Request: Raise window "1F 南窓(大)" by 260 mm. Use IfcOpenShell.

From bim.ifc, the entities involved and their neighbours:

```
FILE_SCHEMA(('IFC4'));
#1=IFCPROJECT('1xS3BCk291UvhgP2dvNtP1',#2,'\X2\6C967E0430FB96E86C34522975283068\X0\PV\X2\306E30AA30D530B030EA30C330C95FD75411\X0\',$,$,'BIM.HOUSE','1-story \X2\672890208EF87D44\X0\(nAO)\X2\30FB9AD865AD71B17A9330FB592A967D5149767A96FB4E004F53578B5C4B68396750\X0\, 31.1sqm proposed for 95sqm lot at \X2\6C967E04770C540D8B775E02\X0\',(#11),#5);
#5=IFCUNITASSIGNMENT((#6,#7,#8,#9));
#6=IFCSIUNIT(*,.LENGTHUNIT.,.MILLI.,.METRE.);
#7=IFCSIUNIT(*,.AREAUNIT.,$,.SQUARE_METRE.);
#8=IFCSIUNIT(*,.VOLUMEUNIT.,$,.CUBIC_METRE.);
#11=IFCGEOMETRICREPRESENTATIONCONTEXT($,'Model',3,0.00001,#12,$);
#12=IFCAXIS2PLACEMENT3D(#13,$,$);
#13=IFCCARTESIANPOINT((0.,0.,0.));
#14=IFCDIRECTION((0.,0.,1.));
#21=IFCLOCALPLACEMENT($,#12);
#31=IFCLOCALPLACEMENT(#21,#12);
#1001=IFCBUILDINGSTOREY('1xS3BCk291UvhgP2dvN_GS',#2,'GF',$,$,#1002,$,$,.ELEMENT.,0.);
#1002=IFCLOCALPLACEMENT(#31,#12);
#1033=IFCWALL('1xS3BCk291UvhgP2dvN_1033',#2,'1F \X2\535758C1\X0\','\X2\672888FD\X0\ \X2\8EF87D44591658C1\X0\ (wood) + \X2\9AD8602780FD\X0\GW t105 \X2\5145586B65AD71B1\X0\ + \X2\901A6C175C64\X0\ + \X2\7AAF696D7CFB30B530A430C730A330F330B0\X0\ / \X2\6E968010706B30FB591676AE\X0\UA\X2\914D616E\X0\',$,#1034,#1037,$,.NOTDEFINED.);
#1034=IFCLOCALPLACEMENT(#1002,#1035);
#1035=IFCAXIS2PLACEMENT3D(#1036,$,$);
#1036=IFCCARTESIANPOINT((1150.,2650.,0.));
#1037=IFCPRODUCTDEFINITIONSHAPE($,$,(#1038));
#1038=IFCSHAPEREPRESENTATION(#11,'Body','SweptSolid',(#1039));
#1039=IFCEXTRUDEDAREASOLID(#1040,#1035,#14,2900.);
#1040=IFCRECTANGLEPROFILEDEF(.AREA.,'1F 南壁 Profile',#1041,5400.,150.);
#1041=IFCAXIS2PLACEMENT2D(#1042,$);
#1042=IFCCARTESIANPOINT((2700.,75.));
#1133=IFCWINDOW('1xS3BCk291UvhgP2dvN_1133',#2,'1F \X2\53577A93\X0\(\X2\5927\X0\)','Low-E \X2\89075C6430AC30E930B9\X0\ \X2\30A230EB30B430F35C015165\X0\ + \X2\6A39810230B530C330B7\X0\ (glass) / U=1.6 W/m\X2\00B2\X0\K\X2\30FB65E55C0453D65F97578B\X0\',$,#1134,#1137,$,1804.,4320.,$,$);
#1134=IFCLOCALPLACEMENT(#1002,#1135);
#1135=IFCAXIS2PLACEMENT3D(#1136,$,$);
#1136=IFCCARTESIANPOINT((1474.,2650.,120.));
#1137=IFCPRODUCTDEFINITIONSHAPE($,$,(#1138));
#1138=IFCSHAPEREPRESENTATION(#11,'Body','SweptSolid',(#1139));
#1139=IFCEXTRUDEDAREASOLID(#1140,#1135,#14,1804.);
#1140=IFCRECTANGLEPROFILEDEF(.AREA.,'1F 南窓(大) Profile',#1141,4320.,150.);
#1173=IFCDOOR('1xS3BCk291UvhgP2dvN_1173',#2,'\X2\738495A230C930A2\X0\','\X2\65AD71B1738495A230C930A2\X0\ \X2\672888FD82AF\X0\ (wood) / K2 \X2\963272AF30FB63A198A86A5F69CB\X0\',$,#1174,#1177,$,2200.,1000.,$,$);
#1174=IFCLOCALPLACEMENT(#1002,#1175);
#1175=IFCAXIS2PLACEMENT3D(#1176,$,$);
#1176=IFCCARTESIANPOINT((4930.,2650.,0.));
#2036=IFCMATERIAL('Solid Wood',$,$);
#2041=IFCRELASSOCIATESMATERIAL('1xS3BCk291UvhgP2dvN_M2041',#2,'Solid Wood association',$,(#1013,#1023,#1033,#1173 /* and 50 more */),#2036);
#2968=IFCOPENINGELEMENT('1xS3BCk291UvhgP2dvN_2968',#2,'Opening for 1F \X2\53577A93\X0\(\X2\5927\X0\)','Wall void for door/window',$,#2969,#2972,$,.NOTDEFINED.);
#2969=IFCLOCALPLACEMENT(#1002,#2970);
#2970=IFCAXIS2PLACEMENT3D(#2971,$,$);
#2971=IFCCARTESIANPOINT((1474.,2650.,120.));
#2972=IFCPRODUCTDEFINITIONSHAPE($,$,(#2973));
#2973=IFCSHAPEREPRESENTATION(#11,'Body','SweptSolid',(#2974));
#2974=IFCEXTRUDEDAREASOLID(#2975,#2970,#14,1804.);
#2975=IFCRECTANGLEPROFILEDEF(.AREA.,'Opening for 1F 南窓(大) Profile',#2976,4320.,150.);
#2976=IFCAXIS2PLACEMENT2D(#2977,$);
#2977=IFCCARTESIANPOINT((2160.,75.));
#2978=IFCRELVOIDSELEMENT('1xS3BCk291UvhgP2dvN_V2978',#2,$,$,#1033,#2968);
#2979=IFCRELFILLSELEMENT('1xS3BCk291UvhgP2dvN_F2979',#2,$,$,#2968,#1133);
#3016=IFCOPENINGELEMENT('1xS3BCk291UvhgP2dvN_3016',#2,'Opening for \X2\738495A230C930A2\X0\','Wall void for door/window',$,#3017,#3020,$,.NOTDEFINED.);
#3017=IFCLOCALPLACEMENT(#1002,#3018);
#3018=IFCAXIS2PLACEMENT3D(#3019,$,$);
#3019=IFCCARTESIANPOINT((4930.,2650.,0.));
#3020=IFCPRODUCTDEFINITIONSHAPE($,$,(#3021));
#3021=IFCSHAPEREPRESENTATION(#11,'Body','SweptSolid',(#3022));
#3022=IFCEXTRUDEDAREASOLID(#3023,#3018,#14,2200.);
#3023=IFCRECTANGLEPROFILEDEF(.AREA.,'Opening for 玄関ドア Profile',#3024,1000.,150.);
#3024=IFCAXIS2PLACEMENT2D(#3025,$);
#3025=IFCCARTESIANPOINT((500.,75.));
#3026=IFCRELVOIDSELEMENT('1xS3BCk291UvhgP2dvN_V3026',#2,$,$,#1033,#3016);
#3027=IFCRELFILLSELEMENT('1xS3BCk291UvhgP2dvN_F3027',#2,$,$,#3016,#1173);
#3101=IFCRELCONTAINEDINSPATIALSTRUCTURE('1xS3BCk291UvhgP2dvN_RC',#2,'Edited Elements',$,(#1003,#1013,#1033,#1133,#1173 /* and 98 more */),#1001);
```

```python
import numpy as np
import ifcopenshell
import ifcopenshell.api.geometry
import ifcopenshell.util.placement
import ifcopenshell.util.unit

model = ifcopenshell.open("bim.ifc")
unit_scale = ifcopenshell.util.unit.calculate_unit_scale(model)

window = model.by_guid("1xS3BCk291UvhgP2dvN_1133")
opening = window.FillsVoids[0].RelatingOpeningElement
dz = 0.26 / unit_scale

shift = np.array([0.0, 0.0, dz])
# The window is not placed relative to its opening, so move both.
for product in (opening, window):
    matrix = ifcopenshell.util.placement.get_local_placement(product.ObjectPlacement)
    matrix[:3, 3] += shift
    ifcopenshell.api.geometry.edit_object_placement(model, product=product, matrix=matrix, is_si=False)

print(f"moved by {dz * unit_scale:+.3f} m")

model.write("bim_edited.ifc")
```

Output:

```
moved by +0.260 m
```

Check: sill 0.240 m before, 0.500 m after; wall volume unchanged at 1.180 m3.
